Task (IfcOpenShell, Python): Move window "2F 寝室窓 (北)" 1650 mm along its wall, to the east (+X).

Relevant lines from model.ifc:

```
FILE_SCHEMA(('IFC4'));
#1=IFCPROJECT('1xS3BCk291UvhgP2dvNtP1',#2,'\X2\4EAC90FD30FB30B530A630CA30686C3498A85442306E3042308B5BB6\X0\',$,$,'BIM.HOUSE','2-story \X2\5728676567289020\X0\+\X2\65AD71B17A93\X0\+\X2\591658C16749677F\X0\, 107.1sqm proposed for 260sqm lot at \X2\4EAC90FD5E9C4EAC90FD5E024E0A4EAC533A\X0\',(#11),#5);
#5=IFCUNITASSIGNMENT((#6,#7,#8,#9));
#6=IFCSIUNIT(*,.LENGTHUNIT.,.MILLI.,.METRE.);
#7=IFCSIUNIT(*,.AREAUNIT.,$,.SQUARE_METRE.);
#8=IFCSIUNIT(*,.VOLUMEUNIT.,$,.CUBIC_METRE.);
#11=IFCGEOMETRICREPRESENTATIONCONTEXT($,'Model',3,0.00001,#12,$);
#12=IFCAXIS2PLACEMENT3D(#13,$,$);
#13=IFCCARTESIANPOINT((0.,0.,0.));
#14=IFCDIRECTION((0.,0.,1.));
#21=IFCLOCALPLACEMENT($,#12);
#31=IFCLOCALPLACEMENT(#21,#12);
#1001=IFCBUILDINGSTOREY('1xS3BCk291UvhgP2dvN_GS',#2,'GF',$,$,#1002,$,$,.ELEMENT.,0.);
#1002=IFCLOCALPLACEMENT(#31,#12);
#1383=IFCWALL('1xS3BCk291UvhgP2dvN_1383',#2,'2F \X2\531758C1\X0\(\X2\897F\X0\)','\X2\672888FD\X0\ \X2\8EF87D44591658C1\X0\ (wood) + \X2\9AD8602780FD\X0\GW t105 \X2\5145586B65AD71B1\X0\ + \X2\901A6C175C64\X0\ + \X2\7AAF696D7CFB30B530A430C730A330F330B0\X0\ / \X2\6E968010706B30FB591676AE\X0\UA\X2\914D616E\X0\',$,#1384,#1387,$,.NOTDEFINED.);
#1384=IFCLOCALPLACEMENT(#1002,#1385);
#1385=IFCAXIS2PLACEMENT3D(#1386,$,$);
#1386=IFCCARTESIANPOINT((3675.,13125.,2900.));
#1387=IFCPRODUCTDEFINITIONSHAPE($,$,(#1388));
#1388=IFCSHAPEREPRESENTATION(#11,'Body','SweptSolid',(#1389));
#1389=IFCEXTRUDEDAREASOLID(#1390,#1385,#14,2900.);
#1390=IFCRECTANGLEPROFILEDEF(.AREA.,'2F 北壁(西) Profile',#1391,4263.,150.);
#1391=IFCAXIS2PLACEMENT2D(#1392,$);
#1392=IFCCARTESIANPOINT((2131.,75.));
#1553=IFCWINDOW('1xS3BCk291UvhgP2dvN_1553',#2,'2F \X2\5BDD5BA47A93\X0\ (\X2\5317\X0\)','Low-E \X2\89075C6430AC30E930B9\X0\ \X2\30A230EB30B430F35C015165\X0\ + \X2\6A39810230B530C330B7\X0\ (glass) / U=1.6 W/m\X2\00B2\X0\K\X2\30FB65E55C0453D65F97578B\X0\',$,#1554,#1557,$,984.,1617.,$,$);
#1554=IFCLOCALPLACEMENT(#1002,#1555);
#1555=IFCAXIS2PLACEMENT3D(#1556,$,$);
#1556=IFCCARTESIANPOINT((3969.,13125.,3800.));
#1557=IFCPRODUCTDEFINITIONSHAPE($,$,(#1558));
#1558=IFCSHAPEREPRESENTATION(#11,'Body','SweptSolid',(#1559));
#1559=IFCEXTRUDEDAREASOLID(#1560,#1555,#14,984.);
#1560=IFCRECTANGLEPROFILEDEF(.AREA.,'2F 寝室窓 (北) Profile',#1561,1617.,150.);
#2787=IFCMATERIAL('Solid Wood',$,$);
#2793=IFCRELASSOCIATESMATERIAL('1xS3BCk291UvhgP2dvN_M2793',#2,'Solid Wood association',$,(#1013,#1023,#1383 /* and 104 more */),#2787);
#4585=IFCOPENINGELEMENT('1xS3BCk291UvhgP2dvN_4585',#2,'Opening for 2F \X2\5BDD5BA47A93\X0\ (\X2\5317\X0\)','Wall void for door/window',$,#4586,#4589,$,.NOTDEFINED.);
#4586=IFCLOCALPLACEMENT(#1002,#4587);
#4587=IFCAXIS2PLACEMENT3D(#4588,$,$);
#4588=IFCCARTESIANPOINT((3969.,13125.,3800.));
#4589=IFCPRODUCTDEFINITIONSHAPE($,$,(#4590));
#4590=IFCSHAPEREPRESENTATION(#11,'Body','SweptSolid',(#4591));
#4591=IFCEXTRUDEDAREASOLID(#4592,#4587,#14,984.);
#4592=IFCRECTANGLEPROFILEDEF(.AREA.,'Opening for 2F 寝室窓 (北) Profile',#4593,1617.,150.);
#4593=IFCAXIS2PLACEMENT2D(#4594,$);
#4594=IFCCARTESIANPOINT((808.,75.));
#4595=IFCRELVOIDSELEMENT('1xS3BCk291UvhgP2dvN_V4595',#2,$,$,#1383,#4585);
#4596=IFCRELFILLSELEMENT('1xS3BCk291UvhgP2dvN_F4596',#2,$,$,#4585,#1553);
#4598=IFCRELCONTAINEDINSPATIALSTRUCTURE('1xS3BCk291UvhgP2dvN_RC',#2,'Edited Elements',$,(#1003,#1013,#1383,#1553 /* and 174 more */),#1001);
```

```python
import ifcopenshell
import ifcopenshell.api.geometry
import ifcopenshell.util.placement

model = ifcopenshell.open("model.ifc")

window = model.by_guid("1xS3BCk291UvhgP2dvN_1553")
opening = window.FillsVoids[0].RelatingOpeningElement
wall = opening.VoidsElements[0].RelatingBuildingElement

wall_matrix = ifcopenshell.util.placement.get_local_placement(wall.ObjectPlacement)
shift = wall_matrix[:3, 0] * 1650.0
before = ifcopenshell.util.placement.get_local_placement(window.ObjectPlacement)[:3, 3].copy()

# The window is not placed relative to its opening, so move both.
for product in (opening, window):
    matrix = ifcopenshell.util.placement.get_local_placement(product.ObjectPlacement)
    matrix[:3, 3] += shift
    ifcopenshell.api.geometry.edit_object_placement(model, product=product, matrix=matrix, is_si=False)

after = ifcopenshell.util.placement.get_local_placement(window.ObjectPlacement)[:3, 3]
print("window moved by", (after - before).round(3) + 0.0)

model.write("model_edited.ifc")
```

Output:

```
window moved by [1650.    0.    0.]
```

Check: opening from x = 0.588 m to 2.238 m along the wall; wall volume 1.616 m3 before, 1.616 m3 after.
